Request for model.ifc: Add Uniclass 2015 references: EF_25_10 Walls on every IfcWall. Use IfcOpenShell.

First a look at what the model holds.

```python
import ifcopenshell

model = ifcopenshell.open("model.ifc")
print(model.schema)
print("classifications:", [c.Name for c in model.by_type("IfcClassification")])
for ifc_class in ("IfcDoor", "IfcRoof", "IfcStair", "IfcWall", "IfcWindow"):
    print(ifc_class, len(model.by_type(ifc_class)))
```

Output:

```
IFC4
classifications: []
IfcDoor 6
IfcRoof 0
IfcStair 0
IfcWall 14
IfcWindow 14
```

```python
import ifcopenshell
import ifcopenshell.api.classification

model = ifcopenshell.open("model.ifc")

system = ifcopenshell.api.classification.add_classification(model, classification="Uniclass 2015")

codes = {
    "IfcWall": ("EF_25_10", "Walls"),
}
for ifc_class, (code, name) in codes.items():
    products = model.by_type(ifc_class)
    ifcopenshell.api.classification.add_reference(
        model, products=products, classification=system, identification=code, name=name
    )
    print(code, len(products))

model.write("model_edited.ifc")
```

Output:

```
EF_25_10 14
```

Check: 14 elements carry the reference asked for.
